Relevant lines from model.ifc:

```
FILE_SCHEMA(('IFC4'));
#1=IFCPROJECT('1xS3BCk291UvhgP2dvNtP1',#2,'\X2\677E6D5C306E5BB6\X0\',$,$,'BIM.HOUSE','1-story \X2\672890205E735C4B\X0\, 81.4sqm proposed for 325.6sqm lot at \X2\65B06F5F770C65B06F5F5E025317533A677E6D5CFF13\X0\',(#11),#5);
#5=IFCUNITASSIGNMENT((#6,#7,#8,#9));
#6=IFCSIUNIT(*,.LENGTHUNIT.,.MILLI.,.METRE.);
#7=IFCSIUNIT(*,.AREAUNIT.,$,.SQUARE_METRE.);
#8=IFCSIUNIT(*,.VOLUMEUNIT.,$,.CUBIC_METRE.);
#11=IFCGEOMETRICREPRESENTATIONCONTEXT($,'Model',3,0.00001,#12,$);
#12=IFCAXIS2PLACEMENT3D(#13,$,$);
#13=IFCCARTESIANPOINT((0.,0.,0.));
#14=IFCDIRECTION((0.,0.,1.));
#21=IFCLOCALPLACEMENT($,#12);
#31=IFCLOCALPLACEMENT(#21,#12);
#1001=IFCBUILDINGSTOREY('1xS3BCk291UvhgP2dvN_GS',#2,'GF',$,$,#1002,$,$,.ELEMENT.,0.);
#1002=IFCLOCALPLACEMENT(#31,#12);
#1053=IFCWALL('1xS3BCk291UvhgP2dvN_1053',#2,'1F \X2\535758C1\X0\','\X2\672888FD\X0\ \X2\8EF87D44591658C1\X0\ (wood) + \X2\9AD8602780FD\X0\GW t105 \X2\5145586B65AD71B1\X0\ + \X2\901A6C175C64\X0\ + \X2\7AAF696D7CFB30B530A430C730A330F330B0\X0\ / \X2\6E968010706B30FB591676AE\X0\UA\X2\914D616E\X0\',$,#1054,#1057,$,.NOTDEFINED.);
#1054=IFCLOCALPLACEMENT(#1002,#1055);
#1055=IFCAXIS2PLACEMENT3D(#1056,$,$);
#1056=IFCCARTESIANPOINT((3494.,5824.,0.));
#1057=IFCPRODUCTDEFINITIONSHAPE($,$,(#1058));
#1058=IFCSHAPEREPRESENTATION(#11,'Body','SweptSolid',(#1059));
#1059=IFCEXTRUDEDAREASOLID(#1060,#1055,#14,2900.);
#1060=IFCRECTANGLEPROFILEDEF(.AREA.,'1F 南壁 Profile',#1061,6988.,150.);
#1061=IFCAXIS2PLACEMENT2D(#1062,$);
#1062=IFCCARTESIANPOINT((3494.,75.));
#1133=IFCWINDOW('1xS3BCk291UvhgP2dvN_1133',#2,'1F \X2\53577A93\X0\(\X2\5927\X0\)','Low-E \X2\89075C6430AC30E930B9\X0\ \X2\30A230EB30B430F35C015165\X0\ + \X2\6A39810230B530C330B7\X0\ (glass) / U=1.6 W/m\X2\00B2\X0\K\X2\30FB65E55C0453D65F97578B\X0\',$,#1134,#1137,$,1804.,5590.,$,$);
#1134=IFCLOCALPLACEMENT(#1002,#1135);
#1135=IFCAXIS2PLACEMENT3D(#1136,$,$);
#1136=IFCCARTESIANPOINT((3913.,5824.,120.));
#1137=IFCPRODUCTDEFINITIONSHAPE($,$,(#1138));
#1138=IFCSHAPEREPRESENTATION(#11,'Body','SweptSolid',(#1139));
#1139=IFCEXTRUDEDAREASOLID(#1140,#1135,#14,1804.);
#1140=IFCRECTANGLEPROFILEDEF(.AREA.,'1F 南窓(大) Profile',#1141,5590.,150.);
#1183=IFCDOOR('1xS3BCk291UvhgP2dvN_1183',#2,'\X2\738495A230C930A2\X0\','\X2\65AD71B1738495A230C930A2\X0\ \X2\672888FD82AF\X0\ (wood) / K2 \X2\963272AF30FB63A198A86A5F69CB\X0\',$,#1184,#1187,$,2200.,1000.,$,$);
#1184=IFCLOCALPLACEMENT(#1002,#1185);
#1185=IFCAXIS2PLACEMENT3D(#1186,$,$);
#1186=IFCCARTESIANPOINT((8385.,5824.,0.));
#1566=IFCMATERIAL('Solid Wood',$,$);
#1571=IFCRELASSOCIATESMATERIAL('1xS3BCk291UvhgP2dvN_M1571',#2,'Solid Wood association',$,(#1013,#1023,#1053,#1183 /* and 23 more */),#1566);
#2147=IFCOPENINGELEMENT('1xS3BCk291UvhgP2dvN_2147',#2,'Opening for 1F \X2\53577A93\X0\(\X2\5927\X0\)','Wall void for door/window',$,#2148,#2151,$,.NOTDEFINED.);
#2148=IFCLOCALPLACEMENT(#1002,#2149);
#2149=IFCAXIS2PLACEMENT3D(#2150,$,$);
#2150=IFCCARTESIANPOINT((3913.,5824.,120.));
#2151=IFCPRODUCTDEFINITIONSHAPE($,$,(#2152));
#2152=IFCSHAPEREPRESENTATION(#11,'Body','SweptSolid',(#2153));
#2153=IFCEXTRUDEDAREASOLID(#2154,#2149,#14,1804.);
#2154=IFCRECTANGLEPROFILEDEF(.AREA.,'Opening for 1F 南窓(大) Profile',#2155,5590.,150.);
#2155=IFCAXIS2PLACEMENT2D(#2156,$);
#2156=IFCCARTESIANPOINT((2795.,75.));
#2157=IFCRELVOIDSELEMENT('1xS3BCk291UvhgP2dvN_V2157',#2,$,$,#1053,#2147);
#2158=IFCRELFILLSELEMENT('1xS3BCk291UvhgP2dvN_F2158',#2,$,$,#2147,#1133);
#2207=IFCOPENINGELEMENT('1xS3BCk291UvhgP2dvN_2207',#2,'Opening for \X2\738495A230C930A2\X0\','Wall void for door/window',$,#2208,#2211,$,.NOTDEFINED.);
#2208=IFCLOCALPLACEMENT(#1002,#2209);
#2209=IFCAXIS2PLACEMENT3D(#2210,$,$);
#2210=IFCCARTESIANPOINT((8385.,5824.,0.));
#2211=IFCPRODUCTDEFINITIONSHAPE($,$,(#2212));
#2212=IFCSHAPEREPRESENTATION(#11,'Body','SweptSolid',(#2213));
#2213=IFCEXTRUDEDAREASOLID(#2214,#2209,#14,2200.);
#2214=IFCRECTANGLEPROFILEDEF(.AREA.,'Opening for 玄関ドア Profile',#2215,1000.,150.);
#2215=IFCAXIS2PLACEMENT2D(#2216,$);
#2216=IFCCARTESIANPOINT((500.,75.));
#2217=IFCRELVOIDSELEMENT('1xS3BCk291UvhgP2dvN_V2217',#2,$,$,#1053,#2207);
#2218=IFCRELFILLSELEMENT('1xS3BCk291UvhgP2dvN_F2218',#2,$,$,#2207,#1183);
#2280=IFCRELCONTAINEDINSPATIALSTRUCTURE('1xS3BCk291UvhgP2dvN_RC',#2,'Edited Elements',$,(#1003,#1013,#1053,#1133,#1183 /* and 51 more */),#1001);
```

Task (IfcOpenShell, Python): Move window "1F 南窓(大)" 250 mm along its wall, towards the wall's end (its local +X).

```python
import ifcopenshell
import ifcopenshell.api.geometry
import ifcopenshell.util.placement
import ifcopenshell.util.unit

model = ifcopenshell.open("model.ifc")
unit_scale = ifcopenshell.util.unit.calculate_unit_scale(model)

window = model.by_guid("1xS3BCk291UvhgP2dvN_1133")
opening = window.FillsVoids[0].RelatingOpeningElement
wall = opening.VoidsElements[0].RelatingBuildingElement

wall_matrix = ifcopenshell.util.placement.get_local_placement(wall.ObjectPlacement)
shift = wall_matrix[:3, 0] * 0.25 / unit_scale
before = ifcopenshell.util.placement.get_local_placement(window.ObjectPlacement)[:3, 3].copy()

# The window is not placed relative to its opening, so move both.
for product in (opening, window):
    matrix = ifcopenshell.util.placement.get_local_placement(product.ObjectPlacement)
    matrix[:3, 3] += shift
    ifcopenshell.api.geometry.edit_object_placement(model, product=product, matrix=matrix, is_si=False)

after = ifcopenshell.util.placement.get_local_placement(window.ObjectPlacement)[:3, 3]
print("window moved by", (after - before).round(3) + 0.0)

model.write("model_updated.ifc")
```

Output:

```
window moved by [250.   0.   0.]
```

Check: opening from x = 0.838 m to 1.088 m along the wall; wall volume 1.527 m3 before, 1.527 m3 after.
